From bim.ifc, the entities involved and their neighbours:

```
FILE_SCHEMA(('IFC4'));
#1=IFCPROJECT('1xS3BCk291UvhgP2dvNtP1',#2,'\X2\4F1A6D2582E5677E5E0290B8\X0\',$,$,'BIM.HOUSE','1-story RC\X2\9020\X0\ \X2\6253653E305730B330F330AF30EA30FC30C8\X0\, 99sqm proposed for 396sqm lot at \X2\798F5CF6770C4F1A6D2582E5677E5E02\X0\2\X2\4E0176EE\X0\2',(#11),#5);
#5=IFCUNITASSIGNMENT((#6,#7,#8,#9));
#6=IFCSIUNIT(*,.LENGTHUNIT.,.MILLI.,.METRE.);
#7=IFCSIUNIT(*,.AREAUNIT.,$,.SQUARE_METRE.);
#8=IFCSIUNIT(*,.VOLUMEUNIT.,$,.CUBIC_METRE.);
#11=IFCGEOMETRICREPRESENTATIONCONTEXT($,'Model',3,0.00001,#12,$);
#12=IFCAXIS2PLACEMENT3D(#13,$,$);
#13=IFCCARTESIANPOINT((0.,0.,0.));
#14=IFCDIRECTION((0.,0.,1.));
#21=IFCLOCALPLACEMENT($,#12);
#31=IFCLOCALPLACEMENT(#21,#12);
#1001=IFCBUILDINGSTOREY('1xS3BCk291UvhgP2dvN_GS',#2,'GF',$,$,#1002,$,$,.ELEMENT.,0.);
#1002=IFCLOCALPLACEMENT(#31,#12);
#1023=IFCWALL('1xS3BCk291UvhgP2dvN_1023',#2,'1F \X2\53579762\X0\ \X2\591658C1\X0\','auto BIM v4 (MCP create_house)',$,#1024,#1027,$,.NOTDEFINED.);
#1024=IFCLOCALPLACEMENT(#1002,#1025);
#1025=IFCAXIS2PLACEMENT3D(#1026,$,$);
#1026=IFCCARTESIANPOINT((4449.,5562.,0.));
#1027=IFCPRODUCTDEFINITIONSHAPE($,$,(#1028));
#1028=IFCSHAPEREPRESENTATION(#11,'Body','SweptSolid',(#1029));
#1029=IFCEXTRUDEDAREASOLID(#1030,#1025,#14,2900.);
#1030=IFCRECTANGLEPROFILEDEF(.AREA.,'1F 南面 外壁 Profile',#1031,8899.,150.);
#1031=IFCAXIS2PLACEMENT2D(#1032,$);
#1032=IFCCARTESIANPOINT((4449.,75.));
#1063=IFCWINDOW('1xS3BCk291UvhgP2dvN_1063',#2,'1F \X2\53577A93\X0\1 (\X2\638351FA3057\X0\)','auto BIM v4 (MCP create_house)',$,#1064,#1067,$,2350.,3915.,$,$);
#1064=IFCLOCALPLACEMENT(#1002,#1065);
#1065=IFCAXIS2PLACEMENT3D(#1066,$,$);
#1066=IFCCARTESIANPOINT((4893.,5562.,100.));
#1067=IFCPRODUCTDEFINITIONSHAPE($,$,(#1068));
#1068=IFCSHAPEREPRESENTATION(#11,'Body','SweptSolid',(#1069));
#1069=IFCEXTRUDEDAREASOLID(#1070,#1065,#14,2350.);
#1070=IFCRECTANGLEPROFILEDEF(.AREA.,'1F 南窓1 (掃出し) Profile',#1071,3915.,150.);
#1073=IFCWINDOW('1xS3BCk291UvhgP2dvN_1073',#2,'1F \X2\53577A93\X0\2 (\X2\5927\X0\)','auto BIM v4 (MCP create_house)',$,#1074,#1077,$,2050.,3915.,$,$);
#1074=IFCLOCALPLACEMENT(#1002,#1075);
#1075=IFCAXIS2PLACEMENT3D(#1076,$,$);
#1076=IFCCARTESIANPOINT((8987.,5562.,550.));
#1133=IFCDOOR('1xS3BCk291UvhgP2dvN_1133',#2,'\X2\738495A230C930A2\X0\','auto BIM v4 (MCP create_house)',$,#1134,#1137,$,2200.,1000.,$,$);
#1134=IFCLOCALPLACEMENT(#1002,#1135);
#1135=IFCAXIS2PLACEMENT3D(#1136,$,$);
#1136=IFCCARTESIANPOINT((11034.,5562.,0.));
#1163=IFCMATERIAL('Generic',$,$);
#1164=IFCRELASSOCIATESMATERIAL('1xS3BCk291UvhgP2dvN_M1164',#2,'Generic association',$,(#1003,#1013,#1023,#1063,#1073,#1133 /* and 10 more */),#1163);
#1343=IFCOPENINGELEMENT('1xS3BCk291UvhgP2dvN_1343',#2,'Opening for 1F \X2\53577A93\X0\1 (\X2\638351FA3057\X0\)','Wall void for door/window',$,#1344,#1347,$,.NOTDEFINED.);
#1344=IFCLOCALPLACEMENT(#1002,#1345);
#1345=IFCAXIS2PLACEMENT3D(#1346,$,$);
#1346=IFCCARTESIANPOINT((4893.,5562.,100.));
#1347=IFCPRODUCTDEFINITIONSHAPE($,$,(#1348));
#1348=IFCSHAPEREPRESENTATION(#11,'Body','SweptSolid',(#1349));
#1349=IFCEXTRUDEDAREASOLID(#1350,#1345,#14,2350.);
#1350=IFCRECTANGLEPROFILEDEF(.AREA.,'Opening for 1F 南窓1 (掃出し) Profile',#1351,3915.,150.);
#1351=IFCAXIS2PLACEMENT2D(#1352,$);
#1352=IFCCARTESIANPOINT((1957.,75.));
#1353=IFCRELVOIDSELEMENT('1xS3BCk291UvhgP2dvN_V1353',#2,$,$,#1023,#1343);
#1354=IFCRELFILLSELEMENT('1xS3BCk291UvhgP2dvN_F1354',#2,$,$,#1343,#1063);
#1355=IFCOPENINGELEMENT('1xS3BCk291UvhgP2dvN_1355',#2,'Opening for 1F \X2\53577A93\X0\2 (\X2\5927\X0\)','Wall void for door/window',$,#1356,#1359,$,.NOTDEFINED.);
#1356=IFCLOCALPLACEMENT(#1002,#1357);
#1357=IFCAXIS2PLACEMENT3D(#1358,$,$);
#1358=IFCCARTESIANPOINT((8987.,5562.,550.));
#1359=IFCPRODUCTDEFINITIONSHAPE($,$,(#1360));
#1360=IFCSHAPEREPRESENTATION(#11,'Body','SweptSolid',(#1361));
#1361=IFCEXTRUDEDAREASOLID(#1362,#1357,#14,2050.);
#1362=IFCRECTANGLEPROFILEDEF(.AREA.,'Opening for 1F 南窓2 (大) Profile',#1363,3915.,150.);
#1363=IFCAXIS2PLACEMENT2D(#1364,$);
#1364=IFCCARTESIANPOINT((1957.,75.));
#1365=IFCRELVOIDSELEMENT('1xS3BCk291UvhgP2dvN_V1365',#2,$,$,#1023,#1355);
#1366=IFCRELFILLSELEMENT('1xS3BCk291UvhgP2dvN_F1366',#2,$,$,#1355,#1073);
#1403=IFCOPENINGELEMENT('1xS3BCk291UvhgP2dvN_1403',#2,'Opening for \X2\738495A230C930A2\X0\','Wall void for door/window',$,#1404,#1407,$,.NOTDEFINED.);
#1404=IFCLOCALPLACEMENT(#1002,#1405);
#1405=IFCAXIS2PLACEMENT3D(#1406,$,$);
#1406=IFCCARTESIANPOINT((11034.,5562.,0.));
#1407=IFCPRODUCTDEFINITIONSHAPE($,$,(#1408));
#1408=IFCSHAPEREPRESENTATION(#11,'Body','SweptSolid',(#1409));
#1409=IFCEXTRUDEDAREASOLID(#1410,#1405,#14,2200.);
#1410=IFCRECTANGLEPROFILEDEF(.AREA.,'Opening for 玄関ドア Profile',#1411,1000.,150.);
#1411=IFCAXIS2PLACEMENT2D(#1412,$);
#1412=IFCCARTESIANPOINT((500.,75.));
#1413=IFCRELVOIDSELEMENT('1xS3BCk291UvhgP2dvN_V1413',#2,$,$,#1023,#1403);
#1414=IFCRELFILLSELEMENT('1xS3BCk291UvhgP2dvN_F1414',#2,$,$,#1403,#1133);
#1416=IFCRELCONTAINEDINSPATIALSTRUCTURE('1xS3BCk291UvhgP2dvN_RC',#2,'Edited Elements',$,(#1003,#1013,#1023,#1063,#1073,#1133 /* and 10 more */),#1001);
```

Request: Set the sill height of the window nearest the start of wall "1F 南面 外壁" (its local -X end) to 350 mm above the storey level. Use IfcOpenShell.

```python
import numpy as np
import ifcopenshell
import ifcopenshell.api.geometry
import ifcopenshell.geom
import ifcopenshell.util.element
import ifcopenshell.util.placement
import ifcopenshell.util.shape
import ifcopenshell.util.unit

model = ifcopenshell.open("bim.ifc")
unit_scale = ifcopenshell.util.unit.calculate_unit_scale(model)

window = model.by_guid("1xS3BCk291UvhgP2dvN_1063")
opening = window.FillsVoids[0].RelatingOpeningElement
storey = ifcopenshell.util.element.get_container(window, ifc_class="IfcBuildingStorey")
level = ifcopenshell.util.placement.get_local_placement(storey.ObjectPlacement)[2, 3]

# The opening's origin need not be at the sill, so measure its lowest point.
shape = ifcopenshell.geom.create_shape(ifcopenshell.geom.settings(), opening)
bottom = ifcopenshell.util.shape.get_shape_bottom_elevation(shape, shape.geometry) / unit_scale
dz = level + 350.0 - bottom

shift = np.array([0.0, 0.0, dz])
# The window is not placed relative to its opening, so move both.
for product in (opening, window):
    matrix = ifcopenshell.util.placement.get_local_placement(product.ObjectPlacement)
    matrix[:3, 3] += shift
    ifcopenshell.api.geometry.edit_object_placement(model, product=product, matrix=matrix, is_si=False)

print(f"moved by {dz * unit_scale:+.3f} m")

model.write("bim-out.ifc")
```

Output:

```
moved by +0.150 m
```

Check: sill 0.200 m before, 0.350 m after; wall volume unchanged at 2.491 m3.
